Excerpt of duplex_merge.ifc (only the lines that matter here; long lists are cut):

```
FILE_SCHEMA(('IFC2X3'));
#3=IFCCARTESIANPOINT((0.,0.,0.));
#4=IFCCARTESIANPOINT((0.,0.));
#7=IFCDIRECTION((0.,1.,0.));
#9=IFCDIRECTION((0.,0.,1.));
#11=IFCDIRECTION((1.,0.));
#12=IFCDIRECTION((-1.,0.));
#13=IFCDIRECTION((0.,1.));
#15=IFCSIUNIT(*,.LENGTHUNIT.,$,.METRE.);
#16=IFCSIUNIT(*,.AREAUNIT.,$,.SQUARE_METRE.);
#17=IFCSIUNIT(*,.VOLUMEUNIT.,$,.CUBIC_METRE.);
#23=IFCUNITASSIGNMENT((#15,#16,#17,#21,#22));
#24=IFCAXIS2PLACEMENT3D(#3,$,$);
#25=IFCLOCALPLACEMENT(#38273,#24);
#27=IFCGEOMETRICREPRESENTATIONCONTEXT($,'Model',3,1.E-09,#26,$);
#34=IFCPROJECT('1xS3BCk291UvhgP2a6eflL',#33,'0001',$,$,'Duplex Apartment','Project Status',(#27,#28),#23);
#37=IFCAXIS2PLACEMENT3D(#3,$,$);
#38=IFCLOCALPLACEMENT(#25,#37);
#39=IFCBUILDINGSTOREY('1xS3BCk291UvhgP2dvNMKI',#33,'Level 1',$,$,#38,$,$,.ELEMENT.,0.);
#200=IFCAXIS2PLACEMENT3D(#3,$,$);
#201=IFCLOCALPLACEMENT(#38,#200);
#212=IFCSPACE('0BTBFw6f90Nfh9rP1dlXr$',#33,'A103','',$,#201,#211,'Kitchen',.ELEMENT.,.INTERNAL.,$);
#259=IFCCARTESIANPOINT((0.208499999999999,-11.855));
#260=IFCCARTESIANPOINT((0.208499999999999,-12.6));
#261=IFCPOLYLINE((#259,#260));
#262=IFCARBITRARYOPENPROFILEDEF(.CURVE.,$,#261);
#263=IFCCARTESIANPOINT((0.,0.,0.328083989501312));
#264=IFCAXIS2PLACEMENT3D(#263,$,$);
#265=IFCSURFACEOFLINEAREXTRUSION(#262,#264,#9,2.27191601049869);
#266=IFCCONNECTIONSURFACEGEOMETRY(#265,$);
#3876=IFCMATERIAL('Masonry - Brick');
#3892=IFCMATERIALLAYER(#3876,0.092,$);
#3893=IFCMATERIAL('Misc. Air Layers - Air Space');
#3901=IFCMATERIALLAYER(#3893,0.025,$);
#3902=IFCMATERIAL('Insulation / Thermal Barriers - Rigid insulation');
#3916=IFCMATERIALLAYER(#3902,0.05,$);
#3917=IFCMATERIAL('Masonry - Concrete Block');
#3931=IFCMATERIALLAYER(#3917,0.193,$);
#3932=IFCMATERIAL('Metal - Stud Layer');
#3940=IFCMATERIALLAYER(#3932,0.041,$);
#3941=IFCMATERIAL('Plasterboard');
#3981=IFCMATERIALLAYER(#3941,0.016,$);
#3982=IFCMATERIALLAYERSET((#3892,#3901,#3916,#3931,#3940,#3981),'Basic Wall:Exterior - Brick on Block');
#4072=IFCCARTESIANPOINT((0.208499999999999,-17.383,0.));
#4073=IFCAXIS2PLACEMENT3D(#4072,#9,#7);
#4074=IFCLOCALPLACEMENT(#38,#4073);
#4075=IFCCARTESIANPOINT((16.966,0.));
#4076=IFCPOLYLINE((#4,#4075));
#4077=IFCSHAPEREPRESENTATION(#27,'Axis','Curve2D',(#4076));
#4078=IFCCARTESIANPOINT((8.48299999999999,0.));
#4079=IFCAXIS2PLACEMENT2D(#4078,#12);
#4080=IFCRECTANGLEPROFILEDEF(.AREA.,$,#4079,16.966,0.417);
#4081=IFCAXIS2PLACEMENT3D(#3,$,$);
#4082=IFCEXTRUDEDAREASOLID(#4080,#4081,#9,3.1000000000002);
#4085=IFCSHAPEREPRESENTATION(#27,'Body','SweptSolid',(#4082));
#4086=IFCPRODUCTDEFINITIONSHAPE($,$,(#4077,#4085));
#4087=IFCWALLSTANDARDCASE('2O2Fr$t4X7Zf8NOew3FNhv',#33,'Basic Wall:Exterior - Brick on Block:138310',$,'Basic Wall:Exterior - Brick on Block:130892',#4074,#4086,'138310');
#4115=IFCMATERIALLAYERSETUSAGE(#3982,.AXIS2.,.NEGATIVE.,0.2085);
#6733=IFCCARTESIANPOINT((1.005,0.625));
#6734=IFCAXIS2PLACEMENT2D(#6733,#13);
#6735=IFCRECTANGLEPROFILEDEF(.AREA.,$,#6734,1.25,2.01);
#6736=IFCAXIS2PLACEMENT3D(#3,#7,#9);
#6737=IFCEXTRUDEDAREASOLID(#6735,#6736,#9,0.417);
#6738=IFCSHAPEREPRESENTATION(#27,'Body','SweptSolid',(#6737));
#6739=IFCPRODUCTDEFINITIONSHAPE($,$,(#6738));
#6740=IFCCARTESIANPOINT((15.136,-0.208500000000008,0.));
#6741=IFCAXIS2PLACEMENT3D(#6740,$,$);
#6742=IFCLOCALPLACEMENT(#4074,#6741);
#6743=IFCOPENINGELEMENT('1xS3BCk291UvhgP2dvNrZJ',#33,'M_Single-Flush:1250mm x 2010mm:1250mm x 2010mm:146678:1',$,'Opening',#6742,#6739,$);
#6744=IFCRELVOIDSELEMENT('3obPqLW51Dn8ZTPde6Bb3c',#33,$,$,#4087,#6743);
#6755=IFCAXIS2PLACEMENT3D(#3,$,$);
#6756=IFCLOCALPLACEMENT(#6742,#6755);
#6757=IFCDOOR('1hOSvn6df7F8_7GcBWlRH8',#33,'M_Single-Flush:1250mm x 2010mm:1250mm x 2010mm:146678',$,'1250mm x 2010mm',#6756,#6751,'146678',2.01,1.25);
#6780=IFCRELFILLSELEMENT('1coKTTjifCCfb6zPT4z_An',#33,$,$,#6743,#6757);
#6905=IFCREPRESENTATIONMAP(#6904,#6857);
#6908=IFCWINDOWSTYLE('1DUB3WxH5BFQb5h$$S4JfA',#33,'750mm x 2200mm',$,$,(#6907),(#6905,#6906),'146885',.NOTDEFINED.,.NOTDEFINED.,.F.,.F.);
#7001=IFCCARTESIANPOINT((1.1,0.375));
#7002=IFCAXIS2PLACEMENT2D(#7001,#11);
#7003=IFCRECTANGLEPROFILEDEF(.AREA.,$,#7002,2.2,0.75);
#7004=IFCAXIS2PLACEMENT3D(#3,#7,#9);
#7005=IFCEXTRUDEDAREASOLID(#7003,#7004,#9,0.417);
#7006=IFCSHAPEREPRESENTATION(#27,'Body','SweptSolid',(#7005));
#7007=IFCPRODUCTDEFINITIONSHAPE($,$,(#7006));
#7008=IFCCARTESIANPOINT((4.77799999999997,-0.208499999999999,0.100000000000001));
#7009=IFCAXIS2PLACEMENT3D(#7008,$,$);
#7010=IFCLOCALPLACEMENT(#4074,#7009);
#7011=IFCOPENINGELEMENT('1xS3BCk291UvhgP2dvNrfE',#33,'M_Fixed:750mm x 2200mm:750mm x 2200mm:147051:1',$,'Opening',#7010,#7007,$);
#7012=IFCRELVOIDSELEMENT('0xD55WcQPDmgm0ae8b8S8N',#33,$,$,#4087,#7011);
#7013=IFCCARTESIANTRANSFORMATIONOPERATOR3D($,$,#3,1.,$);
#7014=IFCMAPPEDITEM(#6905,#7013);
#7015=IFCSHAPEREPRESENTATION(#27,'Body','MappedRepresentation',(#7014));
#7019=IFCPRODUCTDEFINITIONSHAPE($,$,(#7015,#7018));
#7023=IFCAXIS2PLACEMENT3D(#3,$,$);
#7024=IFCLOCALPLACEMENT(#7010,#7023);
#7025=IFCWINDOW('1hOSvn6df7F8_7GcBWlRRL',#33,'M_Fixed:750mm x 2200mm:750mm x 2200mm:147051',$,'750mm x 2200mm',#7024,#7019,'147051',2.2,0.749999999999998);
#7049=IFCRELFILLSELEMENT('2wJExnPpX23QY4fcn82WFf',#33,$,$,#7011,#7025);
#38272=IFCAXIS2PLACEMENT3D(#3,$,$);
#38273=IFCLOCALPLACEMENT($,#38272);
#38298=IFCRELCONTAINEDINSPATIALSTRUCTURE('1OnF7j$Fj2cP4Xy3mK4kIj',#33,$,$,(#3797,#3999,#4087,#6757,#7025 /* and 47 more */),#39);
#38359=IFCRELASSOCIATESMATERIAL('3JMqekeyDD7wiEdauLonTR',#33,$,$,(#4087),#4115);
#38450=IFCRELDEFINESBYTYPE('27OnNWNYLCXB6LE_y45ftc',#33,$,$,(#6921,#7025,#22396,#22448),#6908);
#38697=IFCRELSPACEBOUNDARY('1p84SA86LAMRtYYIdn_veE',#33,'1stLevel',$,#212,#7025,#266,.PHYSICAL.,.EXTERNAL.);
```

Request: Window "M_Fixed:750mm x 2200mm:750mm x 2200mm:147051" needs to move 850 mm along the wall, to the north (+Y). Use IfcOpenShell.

```python
import numpy as np
import ifcopenshell
import ifcopenshell.api.geometry
import ifcopenshell.util.placement
import ifcopenshell.util.unit

model = ifcopenshell.open("duplex_merge.ifc")
unit_scale = ifcopenshell.util.unit.calculate_unit_scale(model)

window = model.by_guid("1hOSvn6df7F8_7GcBWlRRL")
opening = window.FillsVoids[0].RelatingOpeningElement
wall = opening.VoidsElements[0].RelatingBuildingElement

wall_matrix = ifcopenshell.util.placement.get_local_placement(wall.ObjectPlacement)
shift = wall_matrix[:3, 0] * 0.85 / unit_scale
before = ifcopenshell.util.placement.get_local_placement(window.ObjectPlacement)[:3, 3].copy()

# The window is placed relative to its opening, so it follows when the opening moves.
matrix = ifcopenshell.util.placement.get_local_placement(opening.ObjectPlacement)
matrix[:3, 3] += shift
ifcopenshell.api.geometry.edit_object_placement(
    model, product=opening, matrix=matrix, is_si=False, should_transform_children=True
)

# Space boundary surfaces are stored in each space's coordinates; move them too.
for rel in window.ProvidesBoundaries:
    if not rel.ConnectionGeometry:
        continue
    surface = rel.ConnectionGeometry.SurfaceOnRelatingElement
    space_matrix = ifcopenshell.util.placement.get_local_placement(rel.RelatingSpace.ObjectPlacement)
    point = np.array(surface.Position.Location.Coordinates) + space_matrix[:3, :3].T @ shift
    surface.Position = model.createIfcAxis2Placement3D(
        model.createIfcCartesianPoint(point.tolist()), surface.Position.Axis, surface.Position.RefDirection
    )

after = ifcopenshell.util.placement.get_local_placement(window.ObjectPlacement)[:3, 3]
print("window moved by", (after - before).round(3) + 0.0)

model.write("duplex_merge_v2.ifc")
```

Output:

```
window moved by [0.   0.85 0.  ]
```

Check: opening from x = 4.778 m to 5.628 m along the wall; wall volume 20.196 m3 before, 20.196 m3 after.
